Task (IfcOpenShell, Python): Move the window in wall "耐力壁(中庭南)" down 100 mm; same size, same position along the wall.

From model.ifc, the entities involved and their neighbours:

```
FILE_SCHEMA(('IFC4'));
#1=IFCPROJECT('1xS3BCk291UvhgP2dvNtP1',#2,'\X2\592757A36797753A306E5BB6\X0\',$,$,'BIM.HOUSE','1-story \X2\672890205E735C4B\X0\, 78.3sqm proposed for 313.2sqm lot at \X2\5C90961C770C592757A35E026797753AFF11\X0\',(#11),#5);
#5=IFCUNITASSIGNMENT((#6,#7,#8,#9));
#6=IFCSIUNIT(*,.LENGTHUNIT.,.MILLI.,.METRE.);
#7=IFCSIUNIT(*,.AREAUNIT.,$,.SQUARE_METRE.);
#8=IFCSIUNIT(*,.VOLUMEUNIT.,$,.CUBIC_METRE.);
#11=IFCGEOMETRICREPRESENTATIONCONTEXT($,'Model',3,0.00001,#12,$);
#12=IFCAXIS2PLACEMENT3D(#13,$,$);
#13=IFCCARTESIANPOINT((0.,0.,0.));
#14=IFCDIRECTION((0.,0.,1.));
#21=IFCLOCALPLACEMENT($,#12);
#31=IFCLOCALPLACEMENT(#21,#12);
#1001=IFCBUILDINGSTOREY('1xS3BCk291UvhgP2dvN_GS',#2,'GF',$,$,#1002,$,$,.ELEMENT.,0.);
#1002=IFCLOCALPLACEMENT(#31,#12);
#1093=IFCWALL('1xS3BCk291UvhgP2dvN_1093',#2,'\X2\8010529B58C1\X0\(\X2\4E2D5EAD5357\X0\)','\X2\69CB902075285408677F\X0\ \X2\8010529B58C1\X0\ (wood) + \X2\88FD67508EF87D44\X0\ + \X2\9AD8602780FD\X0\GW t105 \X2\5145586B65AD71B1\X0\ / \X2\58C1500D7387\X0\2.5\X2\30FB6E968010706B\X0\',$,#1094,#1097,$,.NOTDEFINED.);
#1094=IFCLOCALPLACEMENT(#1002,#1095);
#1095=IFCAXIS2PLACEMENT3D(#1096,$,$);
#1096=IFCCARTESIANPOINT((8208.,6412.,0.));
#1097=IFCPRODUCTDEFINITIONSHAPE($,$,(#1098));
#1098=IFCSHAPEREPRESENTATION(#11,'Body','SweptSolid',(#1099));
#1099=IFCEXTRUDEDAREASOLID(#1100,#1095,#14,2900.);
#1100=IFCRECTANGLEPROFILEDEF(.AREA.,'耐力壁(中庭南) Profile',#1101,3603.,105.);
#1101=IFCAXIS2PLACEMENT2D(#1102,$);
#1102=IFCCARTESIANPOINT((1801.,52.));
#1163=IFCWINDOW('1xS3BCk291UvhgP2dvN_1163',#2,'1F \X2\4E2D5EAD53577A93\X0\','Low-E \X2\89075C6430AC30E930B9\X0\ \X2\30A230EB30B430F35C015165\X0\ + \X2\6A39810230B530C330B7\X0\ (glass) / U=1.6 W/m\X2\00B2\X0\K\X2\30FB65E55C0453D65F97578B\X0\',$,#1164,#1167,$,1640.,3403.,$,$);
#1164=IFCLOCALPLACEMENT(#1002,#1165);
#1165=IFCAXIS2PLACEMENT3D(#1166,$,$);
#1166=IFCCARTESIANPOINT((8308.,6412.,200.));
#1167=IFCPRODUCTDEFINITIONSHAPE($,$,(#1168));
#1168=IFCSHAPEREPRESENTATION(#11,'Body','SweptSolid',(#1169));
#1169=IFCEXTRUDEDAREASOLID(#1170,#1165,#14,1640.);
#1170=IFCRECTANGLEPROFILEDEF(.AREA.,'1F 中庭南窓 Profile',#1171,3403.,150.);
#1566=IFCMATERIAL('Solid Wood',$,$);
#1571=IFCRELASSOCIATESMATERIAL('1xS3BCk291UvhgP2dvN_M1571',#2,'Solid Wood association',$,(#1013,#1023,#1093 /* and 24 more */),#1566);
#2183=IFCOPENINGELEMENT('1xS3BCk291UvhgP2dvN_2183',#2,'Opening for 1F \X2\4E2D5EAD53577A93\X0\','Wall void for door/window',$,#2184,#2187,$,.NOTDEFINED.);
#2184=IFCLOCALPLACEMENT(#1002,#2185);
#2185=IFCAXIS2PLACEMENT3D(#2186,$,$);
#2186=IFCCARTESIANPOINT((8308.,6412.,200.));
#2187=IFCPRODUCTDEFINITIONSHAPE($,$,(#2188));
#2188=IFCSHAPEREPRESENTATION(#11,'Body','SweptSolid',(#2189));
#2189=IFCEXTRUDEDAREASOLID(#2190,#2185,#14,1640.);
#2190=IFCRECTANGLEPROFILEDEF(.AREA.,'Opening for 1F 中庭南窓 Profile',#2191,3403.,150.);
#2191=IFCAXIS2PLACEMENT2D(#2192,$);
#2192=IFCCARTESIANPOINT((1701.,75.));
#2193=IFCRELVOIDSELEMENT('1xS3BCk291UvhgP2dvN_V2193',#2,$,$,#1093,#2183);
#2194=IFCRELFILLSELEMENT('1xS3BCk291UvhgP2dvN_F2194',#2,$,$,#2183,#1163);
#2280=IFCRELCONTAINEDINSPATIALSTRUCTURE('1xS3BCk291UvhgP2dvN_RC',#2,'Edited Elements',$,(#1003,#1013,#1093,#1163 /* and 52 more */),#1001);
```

```python
import numpy as np
import ifcopenshell
import ifcopenshell.api.geometry
import ifcopenshell.util.placement
import ifcopenshell.util.unit

model = ifcopenshell.open("model.ifc")
unit_scale = ifcopenshell.util.unit.calculate_unit_scale(model)

window = model.by_id(1163)
opening = window.FillsVoids[0].RelatingOpeningElement
dz = -0.1 / unit_scale

shift = np.array([0.0, 0.0, dz])
# The window is not placed relative to its opening, so move both.
for product in (opening, window):
    matrix = ifcopenshell.util.placement.get_local_placement(product.ObjectPlacement)
    matrix[:3, 3] += shift
    ifcopenshell.api.geometry.edit_object_placement(model, product=product, matrix=matrix, is_si=False)

print(f"moved by {dz * unit_scale:+.3f} m")

model.write("model-out.ifc")
```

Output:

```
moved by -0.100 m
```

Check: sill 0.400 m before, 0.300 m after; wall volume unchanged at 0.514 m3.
